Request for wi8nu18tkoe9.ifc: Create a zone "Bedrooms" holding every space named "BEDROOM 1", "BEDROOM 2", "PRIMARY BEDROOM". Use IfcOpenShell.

First a look at what the model holds.

```python
import ifcopenshell

model = ifcopenshell.open("wi8nu18tkoe9.ifc")
print(model.schema)
seen = {}
for space in model.by_type("IfcSpace"):
    seen[space.LongName] = seen.get(space.LongName, 0) + 1
for name, count in sorted(seen.items(), key=str):
    print(count, "x", name)
print("zones:", [z.Name for z in model.by_type("IfcZone")][:20])
```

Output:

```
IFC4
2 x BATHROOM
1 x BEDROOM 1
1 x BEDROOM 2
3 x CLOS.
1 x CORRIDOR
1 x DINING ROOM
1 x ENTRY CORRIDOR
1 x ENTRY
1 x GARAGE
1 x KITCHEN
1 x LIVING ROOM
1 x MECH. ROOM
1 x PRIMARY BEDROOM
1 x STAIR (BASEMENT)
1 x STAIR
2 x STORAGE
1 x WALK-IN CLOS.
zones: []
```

```python
import ifcopenshell
import ifcopenshell.api.group
import ifcopenshell.api.root

model = ifcopenshell.open("wi8nu18tkoe9.ifc")

names = {"BEDROOM 1", "BEDROOM 2", "PRIMARY BEDROOM"}
spaces = [s for s in model.by_type("IfcSpace") if s.LongName in names]

zone = ifcopenshell.api.root.create_entity(model, ifc_class="IfcZone", name="Bedrooms")
ifcopenshell.api.group.assign_group(model, products=spaces, group=zone)
print(len(spaces), "spaces in", zone.Name)

model.write("wi8nu18tkoe9_updated.ifc")
```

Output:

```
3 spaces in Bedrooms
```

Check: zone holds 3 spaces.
